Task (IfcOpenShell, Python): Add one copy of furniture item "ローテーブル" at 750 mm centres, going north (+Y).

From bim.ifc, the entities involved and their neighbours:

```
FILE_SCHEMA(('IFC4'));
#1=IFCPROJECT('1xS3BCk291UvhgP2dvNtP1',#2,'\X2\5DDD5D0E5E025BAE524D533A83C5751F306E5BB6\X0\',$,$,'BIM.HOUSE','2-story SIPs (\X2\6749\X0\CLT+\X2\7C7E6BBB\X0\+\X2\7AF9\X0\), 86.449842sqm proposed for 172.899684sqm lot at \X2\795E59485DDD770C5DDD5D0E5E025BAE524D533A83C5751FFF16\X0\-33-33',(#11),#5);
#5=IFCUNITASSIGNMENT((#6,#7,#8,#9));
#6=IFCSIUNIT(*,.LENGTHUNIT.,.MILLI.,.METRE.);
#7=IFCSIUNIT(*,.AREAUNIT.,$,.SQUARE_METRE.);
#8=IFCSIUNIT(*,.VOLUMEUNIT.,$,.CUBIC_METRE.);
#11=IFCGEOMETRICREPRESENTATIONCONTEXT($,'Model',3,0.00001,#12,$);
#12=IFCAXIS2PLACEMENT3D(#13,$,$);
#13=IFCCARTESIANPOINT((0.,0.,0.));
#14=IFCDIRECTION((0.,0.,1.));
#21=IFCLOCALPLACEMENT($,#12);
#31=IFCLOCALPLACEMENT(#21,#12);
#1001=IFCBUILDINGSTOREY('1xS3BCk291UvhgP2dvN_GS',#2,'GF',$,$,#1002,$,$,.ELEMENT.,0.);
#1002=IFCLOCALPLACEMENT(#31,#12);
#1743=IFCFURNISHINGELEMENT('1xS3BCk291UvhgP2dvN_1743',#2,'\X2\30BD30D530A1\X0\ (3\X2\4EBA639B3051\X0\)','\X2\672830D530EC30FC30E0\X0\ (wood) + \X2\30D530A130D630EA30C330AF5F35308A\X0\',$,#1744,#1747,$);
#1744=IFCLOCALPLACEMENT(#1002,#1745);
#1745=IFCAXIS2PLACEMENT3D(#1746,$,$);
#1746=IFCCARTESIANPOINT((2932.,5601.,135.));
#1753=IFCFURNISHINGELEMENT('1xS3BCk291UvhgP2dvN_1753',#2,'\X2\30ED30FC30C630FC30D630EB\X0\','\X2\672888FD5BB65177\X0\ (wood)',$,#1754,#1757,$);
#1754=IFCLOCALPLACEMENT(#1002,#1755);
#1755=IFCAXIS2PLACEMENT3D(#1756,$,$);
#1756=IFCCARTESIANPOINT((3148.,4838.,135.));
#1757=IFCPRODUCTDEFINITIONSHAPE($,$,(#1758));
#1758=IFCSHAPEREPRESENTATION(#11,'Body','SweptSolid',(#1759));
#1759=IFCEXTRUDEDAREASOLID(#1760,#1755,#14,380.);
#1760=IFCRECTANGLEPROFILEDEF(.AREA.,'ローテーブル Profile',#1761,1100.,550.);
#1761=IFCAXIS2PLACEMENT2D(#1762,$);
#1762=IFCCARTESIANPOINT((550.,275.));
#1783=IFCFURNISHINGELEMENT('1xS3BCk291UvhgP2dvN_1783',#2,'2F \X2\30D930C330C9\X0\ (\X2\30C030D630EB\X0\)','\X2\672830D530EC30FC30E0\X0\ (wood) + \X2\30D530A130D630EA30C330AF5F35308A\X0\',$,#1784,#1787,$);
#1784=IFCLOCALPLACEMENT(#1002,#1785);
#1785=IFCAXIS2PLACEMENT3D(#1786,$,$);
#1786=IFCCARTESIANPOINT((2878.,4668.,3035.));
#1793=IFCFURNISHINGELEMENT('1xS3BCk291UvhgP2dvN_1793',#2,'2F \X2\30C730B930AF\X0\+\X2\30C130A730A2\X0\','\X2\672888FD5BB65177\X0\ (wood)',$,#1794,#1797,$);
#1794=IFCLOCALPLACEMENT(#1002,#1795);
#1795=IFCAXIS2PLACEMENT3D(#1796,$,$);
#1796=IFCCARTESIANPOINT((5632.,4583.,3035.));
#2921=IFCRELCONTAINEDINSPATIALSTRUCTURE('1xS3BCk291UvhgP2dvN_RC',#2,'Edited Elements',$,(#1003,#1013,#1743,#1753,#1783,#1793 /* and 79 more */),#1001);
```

```python
import numpy as np
import ifcopenshell
import ifcopenshell.api.geometry
import ifcopenshell.api.root
import ifcopenshell.util.element
import ifcopenshell.util.placement
import ifcopenshell.util.unit

model = ifcopenshell.open("bim.ifc")
unit_scale = ifcopenshell.util.unit.calculate_unit_scale(model)


def reuse_history(source, copy):
    """copy_class also copies each property set's owner history, people and application; keep the originals."""
    for rel in copy.IsDefinedBy:
        if rel.is_a("IfcRelDefinesByProperties") and (history := rel.RelatingPropertyDefinition.OwnerHistory):
            rel.RelatingPropertyDefinition.OwnerHistory = source.OwnerHistory
            ifcopenshell.util.element.remove_deep2(model, history)


source = model.by_guid("1xS3BCk291UvhgP2dvN_1753")
base = ifcopenshell.util.placement.get_local_placement(source.ObjectPlacement)
step = np.array([0.0, 1.0, 0.0]) * 0.75 / unit_scale

for i in range(1, 2):
    copy = ifcopenshell.api.root.copy_class(model, product=source)
    copy.Representation = ifcopenshell.util.element.copy_deep(
        model, source.Representation, exclude=["IfcGeometricRepresentationContext", "IfcRepresentationMap"]
    )
    reuse_history(source, copy)
    matrix = base.copy()
    matrix[:3, 3] += i * step
    print("added at", matrix[:3, 3].round(3) + 0.0)
    ifcopenshell.api.geometry.edit_object_placement(model, product=copy, matrix=matrix, is_si=False)

model.write("bim-out.ifc")
```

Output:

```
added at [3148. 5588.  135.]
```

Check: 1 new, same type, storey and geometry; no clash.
